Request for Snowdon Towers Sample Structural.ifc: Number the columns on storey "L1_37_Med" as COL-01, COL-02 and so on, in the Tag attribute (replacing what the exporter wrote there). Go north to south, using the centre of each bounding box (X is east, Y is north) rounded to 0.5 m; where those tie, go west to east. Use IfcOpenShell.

First a look at what the model holds.

```python
import ifcopenshell
import ifcopenshell.util.element
import ifcopenshell.util.placement

model = ifcopenshell.open("Snowdon Towers Sample Structural.ifc")
print(model.schema)
storey = next(s for s in model.by_type("IfcBuildingStorey") if s.Name == "L1_37_Med")
columns = [e for e in ifcopenshell.util.element.get_decomposition(storey) if e.is_a("IfcColumn")]
for e in sorted(columns, key=lambda e: e.id()):
    origin = ifcopenshell.util.placement.get_local_placement(e.ObjectPlacement)[:3, 3]
    print(e.id(), e.Tag, e.Name, origin.round(2) + 0.0, sep=" | ")
```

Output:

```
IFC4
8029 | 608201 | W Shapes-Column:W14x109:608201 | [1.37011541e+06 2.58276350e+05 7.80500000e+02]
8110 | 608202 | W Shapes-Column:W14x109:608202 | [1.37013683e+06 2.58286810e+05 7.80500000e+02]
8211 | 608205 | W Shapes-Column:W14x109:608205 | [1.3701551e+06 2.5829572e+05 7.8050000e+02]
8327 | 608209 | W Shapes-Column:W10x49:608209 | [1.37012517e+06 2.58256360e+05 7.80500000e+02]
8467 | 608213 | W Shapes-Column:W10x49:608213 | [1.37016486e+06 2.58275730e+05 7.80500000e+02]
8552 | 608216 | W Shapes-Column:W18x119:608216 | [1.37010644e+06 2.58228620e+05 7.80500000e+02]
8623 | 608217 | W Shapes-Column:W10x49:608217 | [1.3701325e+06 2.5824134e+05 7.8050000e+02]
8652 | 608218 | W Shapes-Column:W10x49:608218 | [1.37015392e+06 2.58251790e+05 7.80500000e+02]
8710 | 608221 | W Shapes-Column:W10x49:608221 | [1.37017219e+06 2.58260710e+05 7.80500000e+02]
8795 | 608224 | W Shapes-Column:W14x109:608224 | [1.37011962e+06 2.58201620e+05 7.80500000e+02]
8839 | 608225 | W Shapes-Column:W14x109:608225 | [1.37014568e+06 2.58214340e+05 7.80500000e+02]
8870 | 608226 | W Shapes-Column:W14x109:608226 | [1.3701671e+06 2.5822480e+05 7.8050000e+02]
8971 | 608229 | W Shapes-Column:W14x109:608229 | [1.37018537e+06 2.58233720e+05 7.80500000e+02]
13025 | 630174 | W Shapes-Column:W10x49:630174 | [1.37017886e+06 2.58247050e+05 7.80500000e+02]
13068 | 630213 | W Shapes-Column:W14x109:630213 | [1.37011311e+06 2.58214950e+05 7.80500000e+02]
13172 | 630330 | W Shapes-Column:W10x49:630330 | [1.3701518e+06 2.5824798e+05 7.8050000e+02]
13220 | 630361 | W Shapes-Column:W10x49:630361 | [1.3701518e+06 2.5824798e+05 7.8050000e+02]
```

```python
import ifcopenshell
import ifcopenshell.geom
import ifcopenshell.util.element
import ifcopenshell.util.shape

model = ifcopenshell.open("Snowdon Towers Sample Structural.ifc")
settings = ifcopenshell.geom.settings()
settings.set("use-world-coords", True)


def centre(element):
    shape = ifcopenshell.geom.create_shape(settings, element)
    return ifcopenshell.util.shape.get_bbox_centroid(shape.geometry)


storey = next(s for s in model.by_type("IfcBuildingStorey") if s.Name == "L1_37_Med")
columns = [e for e in ifcopenshell.util.element.get_decomposition(storey) if e.is_a("IfcColumn")]

# Insertion points can sit at a corner or the storey origin, so sort by the geometry (in metres).
centres = {e: centre(e) for e in columns}
columns.sort(key=lambda e: (-round(centres[e][1] / 0.5), centres[e][0]))

for i, e in enumerate(columns, start=1):
    number = f"COL-{i:02d}"
    e.Tag = number
    print(e.id(), number)

model.write("Snowdon Towers Sample Structural_edited.ifc")
```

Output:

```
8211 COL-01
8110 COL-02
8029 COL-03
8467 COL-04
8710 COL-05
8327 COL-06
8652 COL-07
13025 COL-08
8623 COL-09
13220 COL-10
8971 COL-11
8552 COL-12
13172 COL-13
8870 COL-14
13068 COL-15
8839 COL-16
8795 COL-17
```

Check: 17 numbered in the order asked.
